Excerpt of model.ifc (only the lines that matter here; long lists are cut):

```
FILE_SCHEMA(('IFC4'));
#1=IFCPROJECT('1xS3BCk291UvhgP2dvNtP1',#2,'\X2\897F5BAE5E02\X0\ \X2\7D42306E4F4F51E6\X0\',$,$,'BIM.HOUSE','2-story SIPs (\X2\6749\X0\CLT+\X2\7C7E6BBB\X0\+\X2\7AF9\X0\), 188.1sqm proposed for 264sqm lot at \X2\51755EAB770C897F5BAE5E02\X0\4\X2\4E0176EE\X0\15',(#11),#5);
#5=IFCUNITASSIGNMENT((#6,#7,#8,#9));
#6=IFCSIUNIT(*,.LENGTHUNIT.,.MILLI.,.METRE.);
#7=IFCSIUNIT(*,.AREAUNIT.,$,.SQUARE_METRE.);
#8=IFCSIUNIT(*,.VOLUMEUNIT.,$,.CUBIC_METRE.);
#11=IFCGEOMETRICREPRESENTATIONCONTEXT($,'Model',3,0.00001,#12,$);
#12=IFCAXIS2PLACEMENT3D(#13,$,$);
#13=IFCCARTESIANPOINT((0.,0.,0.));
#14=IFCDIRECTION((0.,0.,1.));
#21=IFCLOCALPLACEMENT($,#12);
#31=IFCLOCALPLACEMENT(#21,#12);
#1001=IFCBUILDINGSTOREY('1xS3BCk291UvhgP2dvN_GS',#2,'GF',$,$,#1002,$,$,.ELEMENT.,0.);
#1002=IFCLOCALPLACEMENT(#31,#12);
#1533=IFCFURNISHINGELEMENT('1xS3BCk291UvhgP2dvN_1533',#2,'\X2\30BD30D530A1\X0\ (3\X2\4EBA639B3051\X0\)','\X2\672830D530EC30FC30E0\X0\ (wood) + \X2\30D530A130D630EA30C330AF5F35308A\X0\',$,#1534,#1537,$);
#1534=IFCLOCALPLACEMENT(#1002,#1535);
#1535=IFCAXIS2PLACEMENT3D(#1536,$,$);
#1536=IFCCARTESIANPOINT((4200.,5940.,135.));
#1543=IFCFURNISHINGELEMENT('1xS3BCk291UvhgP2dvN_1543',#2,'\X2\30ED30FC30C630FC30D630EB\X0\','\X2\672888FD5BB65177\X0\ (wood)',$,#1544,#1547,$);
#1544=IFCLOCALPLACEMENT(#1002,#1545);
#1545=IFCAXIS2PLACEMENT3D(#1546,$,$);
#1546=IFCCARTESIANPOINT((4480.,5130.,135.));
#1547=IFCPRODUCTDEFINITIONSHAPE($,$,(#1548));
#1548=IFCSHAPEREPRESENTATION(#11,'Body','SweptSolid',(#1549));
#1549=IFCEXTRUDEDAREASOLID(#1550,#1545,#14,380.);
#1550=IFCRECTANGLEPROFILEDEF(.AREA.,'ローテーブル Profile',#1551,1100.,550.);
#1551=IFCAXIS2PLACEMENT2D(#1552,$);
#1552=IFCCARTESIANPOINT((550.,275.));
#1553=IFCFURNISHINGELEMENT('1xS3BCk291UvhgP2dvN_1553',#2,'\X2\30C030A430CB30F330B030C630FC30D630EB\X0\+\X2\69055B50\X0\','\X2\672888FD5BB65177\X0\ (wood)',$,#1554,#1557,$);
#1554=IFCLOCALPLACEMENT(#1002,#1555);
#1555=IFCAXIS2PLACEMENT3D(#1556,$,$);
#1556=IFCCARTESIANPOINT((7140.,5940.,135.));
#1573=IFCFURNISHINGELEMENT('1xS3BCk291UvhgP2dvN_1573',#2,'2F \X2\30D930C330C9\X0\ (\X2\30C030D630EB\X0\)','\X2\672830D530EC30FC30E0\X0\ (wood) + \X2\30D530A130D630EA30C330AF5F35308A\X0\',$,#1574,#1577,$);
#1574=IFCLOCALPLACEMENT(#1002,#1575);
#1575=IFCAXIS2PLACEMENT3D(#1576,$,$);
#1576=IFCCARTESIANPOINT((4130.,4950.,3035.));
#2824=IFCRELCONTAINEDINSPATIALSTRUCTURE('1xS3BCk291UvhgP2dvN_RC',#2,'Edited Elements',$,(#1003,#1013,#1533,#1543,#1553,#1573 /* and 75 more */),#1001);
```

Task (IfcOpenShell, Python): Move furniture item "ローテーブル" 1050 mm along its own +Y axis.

```python
import ifcopenshell
import ifcopenshell.api.geometry
import ifcopenshell.util.placement

model = ifcopenshell.open("model.ifc")

item = model.by_id(1543)
matrix = ifcopenshell.util.placement.get_local_placement(item.ObjectPlacement)
matrix[:3, 3] += matrix[:3, 1] * 1050.0
ifcopenshell.api.geometry.edit_object_placement(model, product=item, matrix=matrix, is_si=False)

print(ifcopenshell.util.placement.get_local_placement(item.ObjectPlacement).round(3) + 0.0)

model.write("model_v2.ifc")
```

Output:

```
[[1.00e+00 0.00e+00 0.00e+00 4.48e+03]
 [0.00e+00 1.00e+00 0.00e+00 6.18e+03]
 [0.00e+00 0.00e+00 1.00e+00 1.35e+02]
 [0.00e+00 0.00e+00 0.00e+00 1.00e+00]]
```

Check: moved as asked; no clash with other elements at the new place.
